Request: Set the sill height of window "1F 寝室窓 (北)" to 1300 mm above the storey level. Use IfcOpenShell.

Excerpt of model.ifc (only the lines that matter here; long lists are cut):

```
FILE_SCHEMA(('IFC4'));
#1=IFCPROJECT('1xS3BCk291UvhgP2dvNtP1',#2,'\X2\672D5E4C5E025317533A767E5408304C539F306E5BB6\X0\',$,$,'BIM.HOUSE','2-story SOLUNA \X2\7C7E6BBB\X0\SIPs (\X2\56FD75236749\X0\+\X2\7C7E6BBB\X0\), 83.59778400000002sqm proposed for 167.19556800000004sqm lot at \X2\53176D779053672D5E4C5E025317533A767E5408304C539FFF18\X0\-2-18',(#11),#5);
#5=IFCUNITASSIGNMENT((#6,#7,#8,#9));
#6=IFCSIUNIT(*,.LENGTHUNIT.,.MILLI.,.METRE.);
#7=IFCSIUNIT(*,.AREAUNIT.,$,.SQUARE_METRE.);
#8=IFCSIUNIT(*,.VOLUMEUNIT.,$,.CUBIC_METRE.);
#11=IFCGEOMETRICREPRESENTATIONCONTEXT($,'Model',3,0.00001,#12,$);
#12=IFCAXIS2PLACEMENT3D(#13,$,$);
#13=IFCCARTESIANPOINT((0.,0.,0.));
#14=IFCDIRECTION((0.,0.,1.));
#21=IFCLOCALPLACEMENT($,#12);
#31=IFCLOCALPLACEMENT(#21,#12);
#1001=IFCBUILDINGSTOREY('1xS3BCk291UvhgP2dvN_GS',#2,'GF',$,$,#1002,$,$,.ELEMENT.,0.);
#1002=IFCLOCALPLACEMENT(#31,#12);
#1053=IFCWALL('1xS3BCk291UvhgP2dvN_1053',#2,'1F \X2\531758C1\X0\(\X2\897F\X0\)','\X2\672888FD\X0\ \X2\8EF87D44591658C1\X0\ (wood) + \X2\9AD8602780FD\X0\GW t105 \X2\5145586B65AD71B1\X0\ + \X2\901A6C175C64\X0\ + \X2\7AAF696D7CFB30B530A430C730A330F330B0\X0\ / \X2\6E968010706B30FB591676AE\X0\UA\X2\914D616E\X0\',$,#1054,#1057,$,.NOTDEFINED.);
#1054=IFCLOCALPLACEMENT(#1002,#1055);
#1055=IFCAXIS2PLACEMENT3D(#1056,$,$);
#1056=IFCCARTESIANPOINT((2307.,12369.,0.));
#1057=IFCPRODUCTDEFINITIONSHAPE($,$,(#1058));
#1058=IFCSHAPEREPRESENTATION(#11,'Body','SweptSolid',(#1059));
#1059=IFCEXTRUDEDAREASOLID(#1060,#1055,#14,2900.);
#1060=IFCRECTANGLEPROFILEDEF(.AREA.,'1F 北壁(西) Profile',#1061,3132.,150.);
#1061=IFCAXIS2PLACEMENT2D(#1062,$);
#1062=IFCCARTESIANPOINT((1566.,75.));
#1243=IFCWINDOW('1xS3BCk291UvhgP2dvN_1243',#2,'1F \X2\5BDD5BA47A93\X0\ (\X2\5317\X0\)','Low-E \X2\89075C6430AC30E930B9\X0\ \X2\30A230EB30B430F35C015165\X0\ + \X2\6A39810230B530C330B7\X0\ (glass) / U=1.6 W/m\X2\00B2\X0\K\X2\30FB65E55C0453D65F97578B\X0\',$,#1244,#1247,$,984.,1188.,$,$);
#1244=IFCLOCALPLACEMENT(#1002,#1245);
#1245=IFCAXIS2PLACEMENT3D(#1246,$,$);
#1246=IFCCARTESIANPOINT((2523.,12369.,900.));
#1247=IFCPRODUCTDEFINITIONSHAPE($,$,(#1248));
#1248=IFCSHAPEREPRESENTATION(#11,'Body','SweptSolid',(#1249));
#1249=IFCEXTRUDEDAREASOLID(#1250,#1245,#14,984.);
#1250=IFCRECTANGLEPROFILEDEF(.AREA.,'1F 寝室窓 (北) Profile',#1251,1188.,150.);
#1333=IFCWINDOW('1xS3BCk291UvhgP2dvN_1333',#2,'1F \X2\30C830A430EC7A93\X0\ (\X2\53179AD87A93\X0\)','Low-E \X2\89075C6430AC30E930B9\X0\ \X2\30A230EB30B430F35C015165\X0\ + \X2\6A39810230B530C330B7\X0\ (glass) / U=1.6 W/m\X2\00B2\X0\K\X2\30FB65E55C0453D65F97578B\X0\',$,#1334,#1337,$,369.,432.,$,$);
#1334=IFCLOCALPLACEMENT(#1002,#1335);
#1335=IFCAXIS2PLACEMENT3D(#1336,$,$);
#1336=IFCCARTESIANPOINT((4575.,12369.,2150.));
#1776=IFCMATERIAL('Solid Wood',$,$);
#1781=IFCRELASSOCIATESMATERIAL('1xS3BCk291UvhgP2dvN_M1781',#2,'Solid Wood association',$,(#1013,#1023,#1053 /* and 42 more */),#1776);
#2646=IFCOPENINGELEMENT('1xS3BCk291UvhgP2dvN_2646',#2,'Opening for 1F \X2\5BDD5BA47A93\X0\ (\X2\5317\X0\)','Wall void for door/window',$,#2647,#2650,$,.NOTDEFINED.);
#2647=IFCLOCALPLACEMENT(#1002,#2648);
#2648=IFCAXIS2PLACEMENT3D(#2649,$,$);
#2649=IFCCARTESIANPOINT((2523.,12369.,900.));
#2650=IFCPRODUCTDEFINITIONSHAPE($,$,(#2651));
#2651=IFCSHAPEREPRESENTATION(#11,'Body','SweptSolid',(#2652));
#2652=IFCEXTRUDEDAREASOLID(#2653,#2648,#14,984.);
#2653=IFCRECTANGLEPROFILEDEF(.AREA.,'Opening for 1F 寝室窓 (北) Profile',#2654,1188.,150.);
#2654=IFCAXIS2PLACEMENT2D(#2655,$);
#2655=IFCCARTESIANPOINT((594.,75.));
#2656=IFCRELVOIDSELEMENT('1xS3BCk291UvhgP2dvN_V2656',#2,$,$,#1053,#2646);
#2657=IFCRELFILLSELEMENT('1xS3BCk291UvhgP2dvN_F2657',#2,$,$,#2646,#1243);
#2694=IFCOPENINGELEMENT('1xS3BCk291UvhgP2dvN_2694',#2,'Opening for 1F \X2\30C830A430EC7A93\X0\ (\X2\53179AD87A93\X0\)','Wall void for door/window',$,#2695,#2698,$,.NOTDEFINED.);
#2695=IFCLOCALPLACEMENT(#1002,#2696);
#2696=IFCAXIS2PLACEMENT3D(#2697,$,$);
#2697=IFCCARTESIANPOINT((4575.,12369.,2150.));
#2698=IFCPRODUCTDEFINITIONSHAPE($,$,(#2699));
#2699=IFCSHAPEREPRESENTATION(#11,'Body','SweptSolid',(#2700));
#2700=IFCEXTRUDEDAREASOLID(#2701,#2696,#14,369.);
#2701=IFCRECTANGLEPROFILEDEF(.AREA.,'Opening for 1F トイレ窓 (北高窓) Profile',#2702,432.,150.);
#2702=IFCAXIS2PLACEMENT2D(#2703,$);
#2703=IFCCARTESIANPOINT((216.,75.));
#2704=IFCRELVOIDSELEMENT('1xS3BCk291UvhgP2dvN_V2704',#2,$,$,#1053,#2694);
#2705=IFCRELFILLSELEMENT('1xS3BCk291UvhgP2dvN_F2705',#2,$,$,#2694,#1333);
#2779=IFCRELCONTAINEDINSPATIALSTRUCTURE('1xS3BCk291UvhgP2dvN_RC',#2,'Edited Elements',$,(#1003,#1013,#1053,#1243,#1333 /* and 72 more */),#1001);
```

```python
import numpy as np
import ifcopenshell
import ifcopenshell.api.geometry
import ifcopenshell.geom
import ifcopenshell.util.element
import ifcopenshell.util.placement
import ifcopenshell.util.shape
import ifcopenshell.util.unit

model = ifcopenshell.open("model.ifc")
unit_scale = ifcopenshell.util.unit.calculate_unit_scale(model)

window = model.by_id(1243)
opening = window.FillsVoids[0].RelatingOpeningElement
storey = ifcopenshell.util.element.get_container(window, ifc_class="IfcBuildingStorey")
level = ifcopenshell.util.placement.get_local_placement(storey.ObjectPlacement)[2, 3]

# The opening's origin need not be at the sill, so measure its lowest point.
shape = ifcopenshell.geom.create_shape(ifcopenshell.geom.settings(), opening)
bottom = ifcopenshell.util.shape.get_shape_bottom_elevation(shape, shape.geometry) / unit_scale
dz = level + 1.3 / unit_scale - bottom

shift = np.array([0.0, 0.0, dz])
# The window is not placed relative to its opening, so move both.
for product in (opening, window):
    matrix = ifcopenshell.util.placement.get_local_placement(product.ObjectPlacement)
    matrix[:3, 3] += shift
    ifcopenshell.api.geometry.edit_object_placement(model, product=product, matrix=matrix, is_si=False)

print(f"moved by {dz * unit_scale:+.3f} m")

model.write("model_edited.ifc")
```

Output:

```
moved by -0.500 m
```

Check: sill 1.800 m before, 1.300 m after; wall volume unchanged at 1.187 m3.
